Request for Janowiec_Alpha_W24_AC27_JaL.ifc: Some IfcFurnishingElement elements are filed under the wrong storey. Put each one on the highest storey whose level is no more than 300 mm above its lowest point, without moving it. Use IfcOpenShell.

First a look at what the model holds.

```python
import ifcopenshell
import ifcopenshell.util.element
import ifcopenshell.util.placement

model = ifcopenshell.open("Janowiec_Alpha_W24_AC27_JaL.ifc")
print(model.schema)
for storey in model.by_type("IfcBuildingStorey"):
    level = ifcopenshell.util.placement.get_storey_elevation(storey)
    count = sum(e.is_a("IfcFurnishingElement") for e in ifcopenshell.util.element.get_contained(storey))
    print(storey.id(), storey.Name, round(level, 3), count, sep=" | ")
```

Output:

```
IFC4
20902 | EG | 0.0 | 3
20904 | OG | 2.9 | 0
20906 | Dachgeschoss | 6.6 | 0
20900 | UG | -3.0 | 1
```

```python
import ifcopenshell
import ifcopenshell.api.spatial
import ifcopenshell.geom
import ifcopenshell.util.element
import ifcopenshell.util.placement
import ifcopenshell.util.shape
import ifcopenshell.util.unit

model = ifcopenshell.open("Janowiec_Alpha_W24_AC27_JaL.ifc")
unit_scale = ifcopenshell.util.unit.calculate_unit_scale(model)
settings = ifcopenshell.geom.settings()

levels = sorted(
    ((ifcopenshell.util.placement.get_storey_elevation(s) * unit_scale, s) for s in model.by_type("IfcBuildingStorey")),
    key=lambda pair: pair[0],
)

for e in model.by_type("IfcFurnishingElement"):
    current = e.ContainedInStructure[0].RelatingStructure if e.ContainedInStructure else None
    if current is None or not current.is_a("IfcBuildingStorey"):
        continue
    shape = ifcopenshell.geom.create_shape(settings, e)
    bottom = ifcopenshell.util.shape.get_shape_bottom_elevation(shape, shape.geometry)
    below = [s for level, s in levels if level <= bottom + 0.3]
    storey = below[-1] if below else levels[0][1]
    if storey != current:
        # assign_container keeps the world position.
        ifcopenshell.api.spatial.assign_container(model, products=[e], relating_structure=storey)
        print(e.id(), current.Name, "->", storey.Name)

model.write("Janowiec_Alpha_W24_AC27_JaL_edited.ifc")
```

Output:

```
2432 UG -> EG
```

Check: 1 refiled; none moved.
